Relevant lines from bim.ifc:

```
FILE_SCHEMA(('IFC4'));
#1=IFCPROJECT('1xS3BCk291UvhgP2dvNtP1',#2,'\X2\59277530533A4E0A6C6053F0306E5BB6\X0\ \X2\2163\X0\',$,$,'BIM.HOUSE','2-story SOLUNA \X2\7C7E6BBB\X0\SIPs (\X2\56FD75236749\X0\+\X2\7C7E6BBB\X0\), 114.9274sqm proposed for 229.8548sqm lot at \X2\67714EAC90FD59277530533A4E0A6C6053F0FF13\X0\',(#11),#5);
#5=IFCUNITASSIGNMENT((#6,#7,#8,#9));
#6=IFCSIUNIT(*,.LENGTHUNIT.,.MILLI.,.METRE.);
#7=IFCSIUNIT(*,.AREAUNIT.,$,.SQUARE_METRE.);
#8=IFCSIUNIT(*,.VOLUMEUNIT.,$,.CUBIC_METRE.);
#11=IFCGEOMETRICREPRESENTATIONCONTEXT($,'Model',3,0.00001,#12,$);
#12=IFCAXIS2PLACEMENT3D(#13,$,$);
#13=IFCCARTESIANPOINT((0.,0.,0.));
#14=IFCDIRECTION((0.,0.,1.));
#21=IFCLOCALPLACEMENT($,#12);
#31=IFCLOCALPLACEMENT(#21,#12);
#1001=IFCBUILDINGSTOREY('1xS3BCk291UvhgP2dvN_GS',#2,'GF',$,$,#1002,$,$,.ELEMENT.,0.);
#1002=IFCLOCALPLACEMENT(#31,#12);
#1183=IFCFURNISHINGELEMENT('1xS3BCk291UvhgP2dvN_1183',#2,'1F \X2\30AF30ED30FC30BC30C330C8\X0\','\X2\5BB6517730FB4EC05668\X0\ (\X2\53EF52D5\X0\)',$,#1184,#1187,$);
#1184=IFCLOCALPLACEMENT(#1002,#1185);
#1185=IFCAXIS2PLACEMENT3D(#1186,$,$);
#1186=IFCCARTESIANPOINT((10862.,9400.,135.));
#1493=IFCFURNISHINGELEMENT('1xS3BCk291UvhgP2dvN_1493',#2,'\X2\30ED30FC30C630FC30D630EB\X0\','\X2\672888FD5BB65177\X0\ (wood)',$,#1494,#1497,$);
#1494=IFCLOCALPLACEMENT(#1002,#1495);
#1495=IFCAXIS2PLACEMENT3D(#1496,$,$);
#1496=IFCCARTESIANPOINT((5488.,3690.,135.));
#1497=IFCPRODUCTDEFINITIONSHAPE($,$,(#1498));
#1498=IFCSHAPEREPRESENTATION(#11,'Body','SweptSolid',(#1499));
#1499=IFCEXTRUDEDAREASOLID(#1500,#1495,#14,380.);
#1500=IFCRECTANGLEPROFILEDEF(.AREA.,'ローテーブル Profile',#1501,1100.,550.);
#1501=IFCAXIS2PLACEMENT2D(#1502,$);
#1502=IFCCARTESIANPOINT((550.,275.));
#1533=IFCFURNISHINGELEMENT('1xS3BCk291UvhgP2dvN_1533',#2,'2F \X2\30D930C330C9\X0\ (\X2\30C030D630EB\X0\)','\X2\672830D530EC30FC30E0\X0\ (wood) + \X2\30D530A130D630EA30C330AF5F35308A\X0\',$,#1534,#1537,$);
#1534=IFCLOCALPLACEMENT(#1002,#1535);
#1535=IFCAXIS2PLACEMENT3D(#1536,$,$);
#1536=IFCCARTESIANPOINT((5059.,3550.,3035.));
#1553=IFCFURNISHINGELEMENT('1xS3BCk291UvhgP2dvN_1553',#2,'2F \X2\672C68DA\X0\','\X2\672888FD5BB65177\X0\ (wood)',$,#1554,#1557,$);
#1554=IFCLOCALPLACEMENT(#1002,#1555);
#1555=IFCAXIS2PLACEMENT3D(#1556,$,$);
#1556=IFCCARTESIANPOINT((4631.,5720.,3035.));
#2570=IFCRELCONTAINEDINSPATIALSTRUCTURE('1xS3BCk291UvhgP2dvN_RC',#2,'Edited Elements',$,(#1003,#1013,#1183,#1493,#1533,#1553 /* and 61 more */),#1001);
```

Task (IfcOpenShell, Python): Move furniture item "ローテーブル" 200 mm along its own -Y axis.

```python
import ifcopenshell
import ifcopenshell.api.geometry
import ifcopenshell.util.placement
import ifcopenshell.util.unit

model = ifcopenshell.open("bim.ifc")
unit_scale = ifcopenshell.util.unit.calculate_unit_scale(model)

item = model.by_guid("1xS3BCk291UvhgP2dvN_1493")
matrix = ifcopenshell.util.placement.get_local_placement(item.ObjectPlacement)
matrix[:3, 3] -= matrix[:3, 1] * 0.2 / unit_scale
ifcopenshell.api.geometry.edit_object_placement(model, product=item, matrix=matrix, is_si=False)

print(ifcopenshell.util.placement.get_local_placement(item.ObjectPlacement).round(3) + 0.0)

model.write("bim_v2.ifc")
```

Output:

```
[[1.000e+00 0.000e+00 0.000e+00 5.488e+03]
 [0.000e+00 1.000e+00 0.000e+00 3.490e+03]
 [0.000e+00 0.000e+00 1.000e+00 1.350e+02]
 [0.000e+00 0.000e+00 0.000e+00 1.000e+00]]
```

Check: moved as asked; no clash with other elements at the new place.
